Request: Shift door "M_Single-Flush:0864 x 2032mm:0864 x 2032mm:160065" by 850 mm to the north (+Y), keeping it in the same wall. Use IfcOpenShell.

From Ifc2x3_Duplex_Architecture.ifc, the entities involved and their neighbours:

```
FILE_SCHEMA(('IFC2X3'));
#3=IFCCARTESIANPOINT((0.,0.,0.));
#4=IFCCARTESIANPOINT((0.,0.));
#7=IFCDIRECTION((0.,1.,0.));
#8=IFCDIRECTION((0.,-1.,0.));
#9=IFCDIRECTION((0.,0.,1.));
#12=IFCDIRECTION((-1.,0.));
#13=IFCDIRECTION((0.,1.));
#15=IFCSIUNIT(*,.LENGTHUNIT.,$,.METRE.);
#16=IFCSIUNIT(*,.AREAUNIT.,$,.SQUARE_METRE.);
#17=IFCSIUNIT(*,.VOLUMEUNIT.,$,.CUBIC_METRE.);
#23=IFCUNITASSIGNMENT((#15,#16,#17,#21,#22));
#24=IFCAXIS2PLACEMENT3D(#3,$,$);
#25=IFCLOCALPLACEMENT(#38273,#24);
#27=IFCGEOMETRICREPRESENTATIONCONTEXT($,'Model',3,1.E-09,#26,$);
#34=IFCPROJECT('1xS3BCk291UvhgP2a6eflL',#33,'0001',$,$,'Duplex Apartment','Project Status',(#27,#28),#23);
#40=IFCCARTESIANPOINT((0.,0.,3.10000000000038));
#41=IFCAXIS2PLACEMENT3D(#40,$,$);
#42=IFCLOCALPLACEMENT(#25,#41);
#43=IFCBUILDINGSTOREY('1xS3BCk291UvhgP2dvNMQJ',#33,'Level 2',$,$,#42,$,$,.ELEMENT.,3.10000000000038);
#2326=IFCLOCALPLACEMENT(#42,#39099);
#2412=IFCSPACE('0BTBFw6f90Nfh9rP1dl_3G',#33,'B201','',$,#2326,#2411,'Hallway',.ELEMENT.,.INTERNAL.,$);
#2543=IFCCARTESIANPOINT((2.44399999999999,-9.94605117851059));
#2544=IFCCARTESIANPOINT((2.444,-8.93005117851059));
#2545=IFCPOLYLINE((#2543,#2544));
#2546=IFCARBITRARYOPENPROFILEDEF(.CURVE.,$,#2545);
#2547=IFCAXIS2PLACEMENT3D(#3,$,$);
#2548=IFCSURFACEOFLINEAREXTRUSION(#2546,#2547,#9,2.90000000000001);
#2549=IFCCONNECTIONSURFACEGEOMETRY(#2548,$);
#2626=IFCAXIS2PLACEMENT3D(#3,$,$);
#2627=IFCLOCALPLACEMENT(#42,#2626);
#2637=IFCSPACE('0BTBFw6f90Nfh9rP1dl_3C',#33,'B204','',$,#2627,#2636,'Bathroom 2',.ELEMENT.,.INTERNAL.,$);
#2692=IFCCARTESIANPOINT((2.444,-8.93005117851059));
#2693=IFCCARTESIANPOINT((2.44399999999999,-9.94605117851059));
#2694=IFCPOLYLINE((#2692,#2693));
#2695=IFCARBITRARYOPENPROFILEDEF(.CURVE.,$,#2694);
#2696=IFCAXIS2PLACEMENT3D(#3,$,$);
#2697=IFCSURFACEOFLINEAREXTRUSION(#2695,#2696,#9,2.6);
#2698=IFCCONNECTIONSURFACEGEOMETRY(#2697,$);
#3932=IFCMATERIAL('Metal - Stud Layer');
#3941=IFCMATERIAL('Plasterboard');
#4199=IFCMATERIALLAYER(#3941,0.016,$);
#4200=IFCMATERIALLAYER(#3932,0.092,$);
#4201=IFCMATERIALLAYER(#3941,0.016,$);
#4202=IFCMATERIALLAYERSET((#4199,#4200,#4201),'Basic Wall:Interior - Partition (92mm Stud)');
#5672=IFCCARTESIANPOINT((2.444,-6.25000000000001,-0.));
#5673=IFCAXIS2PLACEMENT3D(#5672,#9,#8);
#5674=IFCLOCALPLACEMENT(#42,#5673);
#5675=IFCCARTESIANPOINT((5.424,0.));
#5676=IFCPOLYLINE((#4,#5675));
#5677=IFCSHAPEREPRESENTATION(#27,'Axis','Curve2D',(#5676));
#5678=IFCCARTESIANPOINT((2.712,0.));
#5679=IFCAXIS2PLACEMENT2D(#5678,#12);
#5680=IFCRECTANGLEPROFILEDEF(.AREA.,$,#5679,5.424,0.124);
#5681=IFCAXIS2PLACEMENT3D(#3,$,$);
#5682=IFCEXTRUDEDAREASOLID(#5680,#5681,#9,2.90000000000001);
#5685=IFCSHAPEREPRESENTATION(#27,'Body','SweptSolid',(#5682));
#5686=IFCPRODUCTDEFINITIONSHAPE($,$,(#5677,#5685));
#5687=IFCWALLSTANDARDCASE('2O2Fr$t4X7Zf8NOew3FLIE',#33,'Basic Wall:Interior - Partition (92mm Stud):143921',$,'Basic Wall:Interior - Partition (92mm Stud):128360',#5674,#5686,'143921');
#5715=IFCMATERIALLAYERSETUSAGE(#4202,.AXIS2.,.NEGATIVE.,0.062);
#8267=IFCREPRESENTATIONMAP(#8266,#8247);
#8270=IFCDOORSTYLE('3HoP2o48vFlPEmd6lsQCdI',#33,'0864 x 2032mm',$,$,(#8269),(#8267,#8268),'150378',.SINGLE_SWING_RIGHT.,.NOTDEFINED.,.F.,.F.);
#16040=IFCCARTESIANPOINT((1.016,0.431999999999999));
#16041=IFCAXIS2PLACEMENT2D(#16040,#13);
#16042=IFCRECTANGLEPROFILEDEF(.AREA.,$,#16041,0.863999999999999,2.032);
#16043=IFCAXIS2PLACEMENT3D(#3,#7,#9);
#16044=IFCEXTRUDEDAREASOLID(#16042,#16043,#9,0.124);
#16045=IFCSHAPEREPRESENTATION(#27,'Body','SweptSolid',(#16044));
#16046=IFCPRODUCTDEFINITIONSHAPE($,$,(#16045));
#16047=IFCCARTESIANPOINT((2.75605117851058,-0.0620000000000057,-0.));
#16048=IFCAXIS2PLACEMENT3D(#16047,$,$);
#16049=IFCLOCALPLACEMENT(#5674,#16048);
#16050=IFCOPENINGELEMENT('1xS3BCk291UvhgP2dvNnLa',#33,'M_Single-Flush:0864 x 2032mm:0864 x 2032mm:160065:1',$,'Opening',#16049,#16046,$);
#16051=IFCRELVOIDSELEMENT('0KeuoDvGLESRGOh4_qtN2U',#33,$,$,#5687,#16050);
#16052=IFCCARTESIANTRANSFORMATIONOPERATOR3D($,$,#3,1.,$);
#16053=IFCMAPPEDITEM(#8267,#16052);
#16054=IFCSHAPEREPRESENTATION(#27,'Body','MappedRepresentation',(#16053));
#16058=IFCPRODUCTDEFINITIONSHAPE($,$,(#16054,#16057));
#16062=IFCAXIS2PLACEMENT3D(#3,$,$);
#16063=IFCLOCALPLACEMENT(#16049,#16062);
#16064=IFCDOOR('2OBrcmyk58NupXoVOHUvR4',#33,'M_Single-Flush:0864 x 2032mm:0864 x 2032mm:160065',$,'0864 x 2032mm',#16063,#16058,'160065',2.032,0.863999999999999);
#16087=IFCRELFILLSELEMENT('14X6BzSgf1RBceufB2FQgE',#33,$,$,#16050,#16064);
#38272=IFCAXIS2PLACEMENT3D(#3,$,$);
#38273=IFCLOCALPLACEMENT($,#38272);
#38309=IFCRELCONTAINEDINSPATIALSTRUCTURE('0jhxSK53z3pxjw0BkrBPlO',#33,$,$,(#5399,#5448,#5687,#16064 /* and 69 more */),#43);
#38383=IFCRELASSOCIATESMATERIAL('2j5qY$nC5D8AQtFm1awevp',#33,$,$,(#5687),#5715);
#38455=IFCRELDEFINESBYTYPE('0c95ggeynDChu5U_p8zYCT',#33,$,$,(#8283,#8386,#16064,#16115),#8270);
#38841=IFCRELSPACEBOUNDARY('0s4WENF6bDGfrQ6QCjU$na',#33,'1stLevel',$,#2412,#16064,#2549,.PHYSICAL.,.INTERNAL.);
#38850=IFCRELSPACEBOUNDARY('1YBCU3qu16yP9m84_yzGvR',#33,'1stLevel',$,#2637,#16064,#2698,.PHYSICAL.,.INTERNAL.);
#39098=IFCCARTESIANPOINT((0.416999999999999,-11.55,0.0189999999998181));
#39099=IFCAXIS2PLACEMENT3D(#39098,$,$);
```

```python
import numpy as np
import ifcopenshell
import ifcopenshell.api.geometry
import ifcopenshell.util.placement
import ifcopenshell.util.unit

model = ifcopenshell.open("Ifc2x3_Duplex_Architecture.ifc")
unit_scale = ifcopenshell.util.unit.calculate_unit_scale(model)

door = model.by_guid("2OBrcmyk58NupXoVOHUvR4")
opening = door.FillsVoids[0].RelatingOpeningElement
wall = opening.VoidsElements[0].RelatingBuildingElement

wall_matrix = ifcopenshell.util.placement.get_local_placement(wall.ObjectPlacement)
shift = wall_matrix[:3, 0] * -0.85 / unit_scale
before = ifcopenshell.util.placement.get_local_placement(door.ObjectPlacement)[:3, 3].copy()

# The door is placed relative to its opening, so it follows when the opening moves.
matrix = ifcopenshell.util.placement.get_local_placement(opening.ObjectPlacement)
matrix[:3, 3] += shift
ifcopenshell.api.geometry.edit_object_placement(
    model, product=opening, matrix=matrix, is_si=False, should_transform_children=True
)

# Space boundary surfaces are stored in each space's coordinates; move them too.
for rel in door.ProvidesBoundaries:
    if not rel.ConnectionGeometry:
        continue
    surface = rel.ConnectionGeometry.SurfaceOnRelatingElement
    space_matrix = ifcopenshell.util.placement.get_local_placement(rel.RelatingSpace.ObjectPlacement)
    point = np.array(surface.Position.Location.Coordinates) + space_matrix[:3, :3].T @ shift
    surface.Position = model.createIfcAxis2Placement3D(
        model.createIfcCartesianPoint(point.tolist()), surface.Position.Axis, surface.Position.RefDirection
    )

after = ifcopenshell.util.placement.get_local_placement(door.ObjectPlacement)[:3, 3]
print("door moved by", (after - before).round(3) + 0.0)

model.write("Ifc2x3_Duplex_Architecture-out.ifc")
```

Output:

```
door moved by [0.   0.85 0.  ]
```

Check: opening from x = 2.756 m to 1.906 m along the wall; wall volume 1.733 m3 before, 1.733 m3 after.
